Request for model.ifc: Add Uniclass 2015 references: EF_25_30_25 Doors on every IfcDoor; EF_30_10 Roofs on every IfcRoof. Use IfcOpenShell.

First a look at what the model holds.

```python
import ifcopenshell

model = ifcopenshell.open("model.ifc")
print(model.schema)
print("classifications:", [c.Name for c in model.by_type("IfcClassification")])
for ifc_class in ("IfcDoor", "IfcRoof", "IfcStair", "IfcWall", "IfcWindow"):
    print(ifc_class, len(model.by_type(ifc_class)))
```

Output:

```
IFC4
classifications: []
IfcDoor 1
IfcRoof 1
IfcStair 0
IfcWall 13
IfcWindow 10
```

```python
import ifcopenshell
import ifcopenshell.api.classification

model = ifcopenshell.open("model.ifc")

system = ifcopenshell.api.classification.add_classification(model, classification="Uniclass 2015")

codes = {
    "IfcDoor": ("EF_25_30_25", "Doors"),
    "IfcRoof": ("EF_30_10", "Roofs"),
}
for ifc_class, (code, name) in codes.items():
    products = model.by_type(ifc_class)
    ifcopenshell.api.classification.add_reference(
        model, products=products, classification=system, identification=code, name=name
    )
    print(code, len(products))

model.write("model_edited.ifc")
```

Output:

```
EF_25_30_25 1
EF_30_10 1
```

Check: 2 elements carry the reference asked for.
